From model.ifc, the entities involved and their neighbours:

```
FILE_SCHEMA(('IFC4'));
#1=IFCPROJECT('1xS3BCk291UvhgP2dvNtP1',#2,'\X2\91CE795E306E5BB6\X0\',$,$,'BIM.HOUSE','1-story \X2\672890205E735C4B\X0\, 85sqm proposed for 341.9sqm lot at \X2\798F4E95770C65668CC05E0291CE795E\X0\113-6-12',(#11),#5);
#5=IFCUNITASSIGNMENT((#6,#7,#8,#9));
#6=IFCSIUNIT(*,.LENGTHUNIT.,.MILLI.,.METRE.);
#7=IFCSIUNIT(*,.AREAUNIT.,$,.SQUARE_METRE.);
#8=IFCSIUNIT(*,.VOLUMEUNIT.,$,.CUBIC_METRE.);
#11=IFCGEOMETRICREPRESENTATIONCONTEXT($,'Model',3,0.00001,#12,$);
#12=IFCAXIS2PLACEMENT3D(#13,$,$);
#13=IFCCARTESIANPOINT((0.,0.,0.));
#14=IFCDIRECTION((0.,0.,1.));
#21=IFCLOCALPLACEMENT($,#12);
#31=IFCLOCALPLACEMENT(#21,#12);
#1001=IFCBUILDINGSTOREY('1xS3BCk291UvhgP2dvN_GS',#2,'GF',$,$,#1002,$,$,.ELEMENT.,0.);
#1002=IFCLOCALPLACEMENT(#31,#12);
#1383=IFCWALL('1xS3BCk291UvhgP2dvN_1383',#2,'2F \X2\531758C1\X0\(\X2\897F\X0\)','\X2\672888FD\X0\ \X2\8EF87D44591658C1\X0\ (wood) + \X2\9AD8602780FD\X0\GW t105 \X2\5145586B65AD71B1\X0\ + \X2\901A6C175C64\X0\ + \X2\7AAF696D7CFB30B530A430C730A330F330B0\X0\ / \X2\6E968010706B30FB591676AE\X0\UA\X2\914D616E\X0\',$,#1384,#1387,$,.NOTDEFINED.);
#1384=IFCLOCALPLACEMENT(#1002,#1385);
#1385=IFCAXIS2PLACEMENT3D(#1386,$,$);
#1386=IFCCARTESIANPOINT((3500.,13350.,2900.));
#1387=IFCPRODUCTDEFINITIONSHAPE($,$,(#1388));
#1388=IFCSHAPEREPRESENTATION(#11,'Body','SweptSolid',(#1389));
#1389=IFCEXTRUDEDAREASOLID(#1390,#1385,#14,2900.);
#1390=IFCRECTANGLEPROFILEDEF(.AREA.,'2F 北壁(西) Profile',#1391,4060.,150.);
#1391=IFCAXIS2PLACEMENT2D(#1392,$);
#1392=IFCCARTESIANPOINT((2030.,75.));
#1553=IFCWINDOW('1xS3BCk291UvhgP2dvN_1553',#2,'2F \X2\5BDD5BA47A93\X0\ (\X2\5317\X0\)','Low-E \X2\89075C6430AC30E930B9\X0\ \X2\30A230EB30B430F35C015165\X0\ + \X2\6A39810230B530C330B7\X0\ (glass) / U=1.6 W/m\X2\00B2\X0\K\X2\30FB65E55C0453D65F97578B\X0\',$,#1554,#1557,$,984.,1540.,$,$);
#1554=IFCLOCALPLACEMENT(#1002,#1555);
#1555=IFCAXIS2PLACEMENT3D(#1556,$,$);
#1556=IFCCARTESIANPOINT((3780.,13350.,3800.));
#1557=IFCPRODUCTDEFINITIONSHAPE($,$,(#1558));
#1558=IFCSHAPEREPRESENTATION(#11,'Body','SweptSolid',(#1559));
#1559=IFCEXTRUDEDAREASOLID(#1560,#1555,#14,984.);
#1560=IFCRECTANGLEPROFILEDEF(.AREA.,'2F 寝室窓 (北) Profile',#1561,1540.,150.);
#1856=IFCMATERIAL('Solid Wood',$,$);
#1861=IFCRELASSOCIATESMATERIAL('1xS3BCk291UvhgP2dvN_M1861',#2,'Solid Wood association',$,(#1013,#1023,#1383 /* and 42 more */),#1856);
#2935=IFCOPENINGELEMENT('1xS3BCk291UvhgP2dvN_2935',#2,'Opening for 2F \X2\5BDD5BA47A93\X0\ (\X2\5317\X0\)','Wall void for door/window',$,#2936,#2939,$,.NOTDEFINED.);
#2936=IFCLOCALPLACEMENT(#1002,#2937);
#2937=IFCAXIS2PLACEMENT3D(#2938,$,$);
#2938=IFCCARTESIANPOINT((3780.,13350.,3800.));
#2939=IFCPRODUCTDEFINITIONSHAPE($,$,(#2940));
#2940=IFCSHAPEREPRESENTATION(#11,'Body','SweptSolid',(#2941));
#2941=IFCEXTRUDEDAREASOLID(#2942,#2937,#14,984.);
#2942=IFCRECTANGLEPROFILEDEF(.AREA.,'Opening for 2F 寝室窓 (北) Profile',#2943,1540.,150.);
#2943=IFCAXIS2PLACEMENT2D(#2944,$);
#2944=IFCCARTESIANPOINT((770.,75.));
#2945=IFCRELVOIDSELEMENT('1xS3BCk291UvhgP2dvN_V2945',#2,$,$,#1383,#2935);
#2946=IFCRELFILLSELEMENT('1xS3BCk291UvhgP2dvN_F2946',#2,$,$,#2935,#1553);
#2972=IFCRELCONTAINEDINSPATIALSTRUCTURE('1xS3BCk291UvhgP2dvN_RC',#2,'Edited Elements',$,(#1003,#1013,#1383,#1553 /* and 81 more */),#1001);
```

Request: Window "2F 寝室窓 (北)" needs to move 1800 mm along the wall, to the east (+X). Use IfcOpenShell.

```python
import ifcopenshell
import ifcopenshell.api.geometry
import ifcopenshell.util.placement

model = ifcopenshell.open("model.ifc")

window = model.by_id(1553)
opening = window.FillsVoids[0].RelatingOpeningElement
wall = opening.VoidsElements[0].RelatingBuildingElement

wall_matrix = ifcopenshell.util.placement.get_local_placement(wall.ObjectPlacement)
shift = wall_matrix[:3, 0] * 1800.0
before = ifcopenshell.util.placement.get_local_placement(window.ObjectPlacement)[:3, 3].copy()

# The window is not placed relative to its opening, so move both.
for product in (opening, window):
    matrix = ifcopenshell.util.placement.get_local_placement(product.ObjectPlacement)
    matrix[:3, 3] += shift
    ifcopenshell.api.geometry.edit_object_placement(model, product=product, matrix=matrix, is_si=False)

after = ifcopenshell.util.placement.get_local_placement(window.ObjectPlacement)[:3, 3]
print("window moved by", (after - before).round(3) + 0.0)

model.write("model_updated.ifc")
```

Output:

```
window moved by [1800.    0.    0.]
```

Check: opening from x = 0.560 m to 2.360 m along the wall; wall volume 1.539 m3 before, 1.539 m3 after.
